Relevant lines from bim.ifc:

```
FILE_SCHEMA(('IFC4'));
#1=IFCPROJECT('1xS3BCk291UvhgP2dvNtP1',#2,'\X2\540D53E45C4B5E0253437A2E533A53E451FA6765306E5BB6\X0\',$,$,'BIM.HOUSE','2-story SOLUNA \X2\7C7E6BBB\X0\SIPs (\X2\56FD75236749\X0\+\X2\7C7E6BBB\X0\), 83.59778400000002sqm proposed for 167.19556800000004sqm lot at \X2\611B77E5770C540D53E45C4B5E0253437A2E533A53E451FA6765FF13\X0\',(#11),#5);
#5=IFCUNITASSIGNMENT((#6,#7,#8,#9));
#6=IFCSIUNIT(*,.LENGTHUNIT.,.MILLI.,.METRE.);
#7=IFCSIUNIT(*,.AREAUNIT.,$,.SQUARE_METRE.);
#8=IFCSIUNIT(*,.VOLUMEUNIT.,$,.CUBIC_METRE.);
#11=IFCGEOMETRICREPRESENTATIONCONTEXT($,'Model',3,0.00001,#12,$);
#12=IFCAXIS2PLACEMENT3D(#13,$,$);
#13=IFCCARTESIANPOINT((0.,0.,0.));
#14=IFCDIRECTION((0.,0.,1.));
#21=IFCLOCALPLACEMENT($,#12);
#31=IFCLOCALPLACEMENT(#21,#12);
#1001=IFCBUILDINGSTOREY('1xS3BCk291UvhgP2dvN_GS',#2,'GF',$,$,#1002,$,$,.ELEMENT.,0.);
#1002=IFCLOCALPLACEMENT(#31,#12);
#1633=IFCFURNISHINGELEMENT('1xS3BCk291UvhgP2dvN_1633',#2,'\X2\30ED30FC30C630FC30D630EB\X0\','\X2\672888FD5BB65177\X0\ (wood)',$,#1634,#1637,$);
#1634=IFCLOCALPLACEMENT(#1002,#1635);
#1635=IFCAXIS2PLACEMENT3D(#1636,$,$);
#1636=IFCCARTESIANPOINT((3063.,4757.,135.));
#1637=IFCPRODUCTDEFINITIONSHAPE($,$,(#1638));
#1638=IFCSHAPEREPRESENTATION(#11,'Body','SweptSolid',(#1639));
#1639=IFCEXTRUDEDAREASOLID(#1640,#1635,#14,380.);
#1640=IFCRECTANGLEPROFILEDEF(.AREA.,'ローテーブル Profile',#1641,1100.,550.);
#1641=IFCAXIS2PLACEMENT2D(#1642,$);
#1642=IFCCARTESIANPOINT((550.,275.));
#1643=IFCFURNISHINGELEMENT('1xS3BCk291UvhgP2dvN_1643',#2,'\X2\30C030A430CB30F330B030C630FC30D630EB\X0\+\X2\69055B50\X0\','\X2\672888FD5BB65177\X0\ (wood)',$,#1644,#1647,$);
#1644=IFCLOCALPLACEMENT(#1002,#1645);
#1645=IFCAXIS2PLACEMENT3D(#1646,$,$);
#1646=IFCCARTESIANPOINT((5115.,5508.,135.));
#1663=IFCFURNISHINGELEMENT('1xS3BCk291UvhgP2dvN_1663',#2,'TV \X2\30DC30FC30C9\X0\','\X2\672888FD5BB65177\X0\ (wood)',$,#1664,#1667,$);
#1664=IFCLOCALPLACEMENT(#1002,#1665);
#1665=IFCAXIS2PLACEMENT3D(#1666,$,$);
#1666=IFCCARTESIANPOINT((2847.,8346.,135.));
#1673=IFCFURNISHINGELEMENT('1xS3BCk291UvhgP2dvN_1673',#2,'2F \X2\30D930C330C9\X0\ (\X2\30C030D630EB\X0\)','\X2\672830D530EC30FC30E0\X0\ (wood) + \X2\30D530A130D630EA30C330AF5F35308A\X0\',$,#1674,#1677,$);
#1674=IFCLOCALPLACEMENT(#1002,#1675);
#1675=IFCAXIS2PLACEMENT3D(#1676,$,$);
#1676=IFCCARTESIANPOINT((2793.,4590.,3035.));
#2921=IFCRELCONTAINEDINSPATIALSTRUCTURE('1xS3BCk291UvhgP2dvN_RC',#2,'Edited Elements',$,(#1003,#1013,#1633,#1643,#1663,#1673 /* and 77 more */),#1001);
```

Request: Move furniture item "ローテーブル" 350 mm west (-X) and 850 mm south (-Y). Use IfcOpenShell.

```python
import ifcopenshell
import ifcopenshell.api.geometry
import ifcopenshell.util.placement
import ifcopenshell.util.unit

model = ifcopenshell.open("bim.ifc")
unit_scale = ifcopenshell.util.unit.calculate_unit_scale(model)

item = model.by_id(1633)
matrix = ifcopenshell.util.placement.get_local_placement(item.ObjectPlacement)
matrix[0, 3] -= 0.35 / unit_scale
matrix[1, 3] -= 0.85 / unit_scale
ifcopenshell.api.geometry.edit_object_placement(model, product=item, matrix=matrix, is_si=False)

print(ifcopenshell.util.placement.get_local_placement(item.ObjectPlacement).round(3) + 0.0)

model.write("bim_v2.ifc")
```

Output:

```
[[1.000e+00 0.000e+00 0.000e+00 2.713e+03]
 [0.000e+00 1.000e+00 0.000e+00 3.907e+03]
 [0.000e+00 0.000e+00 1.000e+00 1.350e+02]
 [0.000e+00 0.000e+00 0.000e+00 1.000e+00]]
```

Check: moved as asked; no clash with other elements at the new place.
